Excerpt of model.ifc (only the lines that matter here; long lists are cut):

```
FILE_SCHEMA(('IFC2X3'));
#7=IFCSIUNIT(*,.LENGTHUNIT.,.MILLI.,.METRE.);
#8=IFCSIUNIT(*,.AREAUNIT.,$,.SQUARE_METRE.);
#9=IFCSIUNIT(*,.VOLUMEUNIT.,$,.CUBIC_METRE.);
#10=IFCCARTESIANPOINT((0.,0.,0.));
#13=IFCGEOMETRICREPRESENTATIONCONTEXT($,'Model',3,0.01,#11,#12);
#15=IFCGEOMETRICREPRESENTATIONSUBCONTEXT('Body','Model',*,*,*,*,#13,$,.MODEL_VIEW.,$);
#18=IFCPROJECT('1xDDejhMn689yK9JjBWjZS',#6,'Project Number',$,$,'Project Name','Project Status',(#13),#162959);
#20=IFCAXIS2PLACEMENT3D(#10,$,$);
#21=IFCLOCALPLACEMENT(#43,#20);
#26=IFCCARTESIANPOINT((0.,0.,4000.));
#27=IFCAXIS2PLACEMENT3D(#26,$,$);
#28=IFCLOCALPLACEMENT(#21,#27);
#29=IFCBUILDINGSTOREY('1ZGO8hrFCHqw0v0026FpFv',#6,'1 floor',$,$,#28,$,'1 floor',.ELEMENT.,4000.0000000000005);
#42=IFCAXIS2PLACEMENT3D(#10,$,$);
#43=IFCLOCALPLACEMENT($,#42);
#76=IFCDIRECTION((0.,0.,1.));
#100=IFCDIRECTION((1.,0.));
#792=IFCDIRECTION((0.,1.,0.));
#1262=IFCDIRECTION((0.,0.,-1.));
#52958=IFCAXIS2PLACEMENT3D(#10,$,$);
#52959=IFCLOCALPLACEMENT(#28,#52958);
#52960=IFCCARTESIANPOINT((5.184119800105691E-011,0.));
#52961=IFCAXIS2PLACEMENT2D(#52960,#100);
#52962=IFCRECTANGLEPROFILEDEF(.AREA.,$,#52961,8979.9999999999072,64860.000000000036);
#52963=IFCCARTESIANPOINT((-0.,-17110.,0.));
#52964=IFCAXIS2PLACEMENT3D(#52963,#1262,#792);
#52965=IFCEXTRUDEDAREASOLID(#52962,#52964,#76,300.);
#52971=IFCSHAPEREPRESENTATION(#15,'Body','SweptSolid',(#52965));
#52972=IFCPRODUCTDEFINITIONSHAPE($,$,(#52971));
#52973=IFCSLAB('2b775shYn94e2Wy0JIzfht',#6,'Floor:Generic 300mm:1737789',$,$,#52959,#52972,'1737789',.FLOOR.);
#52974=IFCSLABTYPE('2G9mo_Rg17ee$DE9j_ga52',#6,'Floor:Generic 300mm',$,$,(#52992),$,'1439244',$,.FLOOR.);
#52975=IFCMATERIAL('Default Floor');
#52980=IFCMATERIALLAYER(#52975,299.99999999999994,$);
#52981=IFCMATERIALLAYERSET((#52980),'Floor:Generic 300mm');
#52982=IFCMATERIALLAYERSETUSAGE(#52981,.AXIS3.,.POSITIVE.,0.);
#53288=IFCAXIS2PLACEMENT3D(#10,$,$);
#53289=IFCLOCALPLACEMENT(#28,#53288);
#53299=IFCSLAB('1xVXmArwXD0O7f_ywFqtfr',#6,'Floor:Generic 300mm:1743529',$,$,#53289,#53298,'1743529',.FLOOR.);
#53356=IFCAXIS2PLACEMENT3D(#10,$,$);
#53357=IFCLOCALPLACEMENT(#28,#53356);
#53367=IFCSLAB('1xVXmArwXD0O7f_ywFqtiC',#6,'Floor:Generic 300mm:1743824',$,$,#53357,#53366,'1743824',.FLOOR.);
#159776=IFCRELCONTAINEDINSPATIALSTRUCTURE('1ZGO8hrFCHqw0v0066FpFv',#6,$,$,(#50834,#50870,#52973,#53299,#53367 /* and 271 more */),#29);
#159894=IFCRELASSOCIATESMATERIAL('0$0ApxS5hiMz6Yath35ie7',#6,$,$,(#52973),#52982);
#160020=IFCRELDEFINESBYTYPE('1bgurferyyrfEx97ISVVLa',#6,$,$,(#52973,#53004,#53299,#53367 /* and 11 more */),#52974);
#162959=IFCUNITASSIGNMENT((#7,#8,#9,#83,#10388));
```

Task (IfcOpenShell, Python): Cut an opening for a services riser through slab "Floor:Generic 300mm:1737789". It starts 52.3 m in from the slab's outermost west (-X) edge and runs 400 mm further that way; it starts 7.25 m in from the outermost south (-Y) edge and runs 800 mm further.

```python
import numpy as np
import ifcopenshell
import ifcopenshell.api.feature
import ifcopenshell.api.geometry
import ifcopenshell.api.root
import ifcopenshell.geom
import ifcopenshell.util.placement
import ifcopenshell.util.representation
import ifcopenshell.util.shape
import ifcopenshell.util.unit

model = ifcopenshell.open("model.ifc")
unit_scale = ifcopenshell.util.unit.calculate_unit_scale(model)
settings = ifcopenshell.geom.settings()


def volume(element):
    """Net volume in cubic metres, openings subtracted."""
    shape = ifcopenshell.geom.create_shape(settings, element)
    return ifcopenshell.util.shape.get_volume(shape.geometry)


slab = model.by_guid("2b775shYn94e2Wy0JIzfht")
before = volume(slab)

# Extent in the slab's own axes, in metres. The edges named are its -X and -Y sides.
slab_shape = ifcopenshell.geom.create_shape(settings, slab)
vertices = ifcopenshell.util.shape.get_vertices(slab_shape.geometry)
x_min, y_min, bottom = vertices.min(axis=0)
top = vertices[:, 2].max()

opening = ifcopenshell.api.root.create_entity(model, ifc_class="IfcOpeningElement", name="Services riser opening")
context = ifcopenshell.util.representation.get_context(model, "Model", "Body", "MODEL_VIEW")
width, depth = 0.4, 0.8
outline = [(0.0, 0.0), (width, 0.0), (width, depth), (0.0, depth), (0.0, 0.0)]
# Overshoot both faces by 50 mm so the cut is clean.
shape = ifcopenshell.api.geometry.add_slab_representation(
    model, context=context, depth=top - bottom + 0.1, polyline=outline
)
ifcopenshell.api.geometry.assign_representation(model, product=opening, representation=shape)

matrix = ifcopenshell.util.placement.get_local_placement(slab.ObjectPlacement)
matrix[:, 3] = matrix @ np.append(np.array([x_min + 52.3, y_min + 7.25, bottom - 0.05]) / unit_scale, 1.0)
ifcopenshell.api.geometry.edit_object_placement(model, product=opening, matrix=matrix, is_si=False)
ifcopenshell.api.feature.add_feature(model, feature=opening, element=slab)

after = volume(slab)

print(f"slab volume {before:.3f} -> {after:.3f} m3")

model.write("model_v2.ifc")
```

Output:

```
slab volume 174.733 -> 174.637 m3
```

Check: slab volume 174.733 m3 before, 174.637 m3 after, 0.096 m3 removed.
